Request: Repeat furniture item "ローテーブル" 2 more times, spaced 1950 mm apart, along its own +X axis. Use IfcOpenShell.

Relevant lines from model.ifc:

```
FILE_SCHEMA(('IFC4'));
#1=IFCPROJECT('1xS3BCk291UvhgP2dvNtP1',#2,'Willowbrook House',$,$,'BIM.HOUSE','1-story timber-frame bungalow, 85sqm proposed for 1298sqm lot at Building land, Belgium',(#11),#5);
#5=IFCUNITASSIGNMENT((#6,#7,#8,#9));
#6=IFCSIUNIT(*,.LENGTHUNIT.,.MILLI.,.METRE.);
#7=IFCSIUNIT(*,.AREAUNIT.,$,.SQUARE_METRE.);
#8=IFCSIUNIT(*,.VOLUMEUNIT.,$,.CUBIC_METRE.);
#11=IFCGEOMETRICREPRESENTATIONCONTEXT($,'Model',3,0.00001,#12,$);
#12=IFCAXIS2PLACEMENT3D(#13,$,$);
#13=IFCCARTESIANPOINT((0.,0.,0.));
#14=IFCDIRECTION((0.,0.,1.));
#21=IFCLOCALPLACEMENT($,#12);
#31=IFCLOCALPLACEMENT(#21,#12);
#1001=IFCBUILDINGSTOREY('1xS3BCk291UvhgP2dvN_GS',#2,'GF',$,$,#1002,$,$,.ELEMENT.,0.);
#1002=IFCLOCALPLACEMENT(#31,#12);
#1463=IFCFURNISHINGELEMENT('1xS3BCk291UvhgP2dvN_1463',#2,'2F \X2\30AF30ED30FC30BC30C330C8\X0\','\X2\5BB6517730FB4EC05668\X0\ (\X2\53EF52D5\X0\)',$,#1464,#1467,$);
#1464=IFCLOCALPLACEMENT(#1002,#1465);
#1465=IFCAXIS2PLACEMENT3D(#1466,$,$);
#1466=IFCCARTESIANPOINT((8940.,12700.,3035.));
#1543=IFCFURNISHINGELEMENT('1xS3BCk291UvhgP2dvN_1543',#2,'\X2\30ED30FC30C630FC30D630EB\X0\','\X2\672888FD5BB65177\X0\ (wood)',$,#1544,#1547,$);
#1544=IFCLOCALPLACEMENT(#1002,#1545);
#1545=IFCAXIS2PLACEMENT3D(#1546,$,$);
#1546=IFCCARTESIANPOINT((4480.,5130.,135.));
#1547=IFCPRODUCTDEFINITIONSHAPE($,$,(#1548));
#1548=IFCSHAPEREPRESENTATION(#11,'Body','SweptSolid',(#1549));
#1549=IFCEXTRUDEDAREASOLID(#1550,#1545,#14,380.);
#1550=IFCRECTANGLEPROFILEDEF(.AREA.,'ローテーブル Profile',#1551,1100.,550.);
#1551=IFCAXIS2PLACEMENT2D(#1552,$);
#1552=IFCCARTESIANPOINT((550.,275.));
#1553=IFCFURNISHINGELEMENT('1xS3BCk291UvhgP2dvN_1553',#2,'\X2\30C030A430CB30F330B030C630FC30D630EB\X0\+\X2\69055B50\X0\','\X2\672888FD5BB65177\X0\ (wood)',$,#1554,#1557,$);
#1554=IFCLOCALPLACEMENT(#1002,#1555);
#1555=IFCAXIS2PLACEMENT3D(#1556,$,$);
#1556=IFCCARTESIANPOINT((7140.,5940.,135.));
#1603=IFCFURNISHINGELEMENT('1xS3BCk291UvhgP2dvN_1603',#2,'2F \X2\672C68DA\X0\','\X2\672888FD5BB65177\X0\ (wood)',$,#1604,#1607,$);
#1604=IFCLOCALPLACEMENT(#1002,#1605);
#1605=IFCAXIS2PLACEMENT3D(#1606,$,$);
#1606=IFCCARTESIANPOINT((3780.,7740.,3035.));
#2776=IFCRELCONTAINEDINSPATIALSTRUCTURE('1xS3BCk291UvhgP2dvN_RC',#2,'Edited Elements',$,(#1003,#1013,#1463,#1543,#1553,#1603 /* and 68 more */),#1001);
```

```python
import ifcopenshell
import ifcopenshell.api.geometry
import ifcopenshell.api.root
import ifcopenshell.util.element
import ifcopenshell.util.placement
import ifcopenshell.util.unit

model = ifcopenshell.open("model.ifc")
unit_scale = ifcopenshell.util.unit.calculate_unit_scale(model)


def reuse_history(source, copy):
    """copy_class also copies each property set's owner history, people and application; keep the originals."""
    for rel in copy.IsDefinedBy:
        if rel.is_a("IfcRelDefinesByProperties") and (history := rel.RelatingPropertyDefinition.OwnerHistory):
            rel.RelatingPropertyDefinition.OwnerHistory = source.OwnerHistory
            ifcopenshell.util.element.remove_deep2(model, history)


source = model.by_id(1543)
base = ifcopenshell.util.placement.get_local_placement(source.ObjectPlacement)
step = base[:3, 0] * 1.95 / unit_scale

for i in range(1, 3):
    copy = ifcopenshell.api.root.copy_class(model, product=source)
    copy.Representation = ifcopenshell.util.element.copy_deep(
        model, source.Representation, exclude=["IfcGeometricRepresentationContext", "IfcRepresentationMap"]
    )
    reuse_history(source, copy)
    matrix = base.copy()
    matrix[:3, 3] += i * step
    print("added at", matrix[:3, 3].round(3) + 0.0)
    ifcopenshell.api.geometry.edit_object_placement(model, product=copy, matrix=matrix, is_si=False)

model.write("model_updated.ifc")
```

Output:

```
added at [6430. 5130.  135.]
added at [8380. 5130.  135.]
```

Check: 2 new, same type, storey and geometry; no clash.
